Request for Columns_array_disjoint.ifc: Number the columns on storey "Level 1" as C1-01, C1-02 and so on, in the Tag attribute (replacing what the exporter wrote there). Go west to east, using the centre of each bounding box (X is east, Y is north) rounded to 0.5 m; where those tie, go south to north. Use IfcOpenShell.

First a look at what the model holds.

```python
import ifcopenshell
import ifcopenshell.util.element
import ifcopenshell.util.placement

model = ifcopenshell.open("Columns_array_disjoint.ifc")
print(model.schema)
storey = next(s for s in model.by_type("IfcBuildingStorey") if s.Name == "Level 1")
columns = [e for e in ifcopenshell.util.element.get_decomposition(storey) if e.is_a("IfcColumn")]
for e in sorted(columns, key=lambda e: e.id()):
    origin = ifcopenshell.util.placement.get_local_placement(e.ObjectPlacement)[:3, 3]
    print(e.id(), e.Tag, e.Name, origin.round(2) + 0.0, sep=" | ")
```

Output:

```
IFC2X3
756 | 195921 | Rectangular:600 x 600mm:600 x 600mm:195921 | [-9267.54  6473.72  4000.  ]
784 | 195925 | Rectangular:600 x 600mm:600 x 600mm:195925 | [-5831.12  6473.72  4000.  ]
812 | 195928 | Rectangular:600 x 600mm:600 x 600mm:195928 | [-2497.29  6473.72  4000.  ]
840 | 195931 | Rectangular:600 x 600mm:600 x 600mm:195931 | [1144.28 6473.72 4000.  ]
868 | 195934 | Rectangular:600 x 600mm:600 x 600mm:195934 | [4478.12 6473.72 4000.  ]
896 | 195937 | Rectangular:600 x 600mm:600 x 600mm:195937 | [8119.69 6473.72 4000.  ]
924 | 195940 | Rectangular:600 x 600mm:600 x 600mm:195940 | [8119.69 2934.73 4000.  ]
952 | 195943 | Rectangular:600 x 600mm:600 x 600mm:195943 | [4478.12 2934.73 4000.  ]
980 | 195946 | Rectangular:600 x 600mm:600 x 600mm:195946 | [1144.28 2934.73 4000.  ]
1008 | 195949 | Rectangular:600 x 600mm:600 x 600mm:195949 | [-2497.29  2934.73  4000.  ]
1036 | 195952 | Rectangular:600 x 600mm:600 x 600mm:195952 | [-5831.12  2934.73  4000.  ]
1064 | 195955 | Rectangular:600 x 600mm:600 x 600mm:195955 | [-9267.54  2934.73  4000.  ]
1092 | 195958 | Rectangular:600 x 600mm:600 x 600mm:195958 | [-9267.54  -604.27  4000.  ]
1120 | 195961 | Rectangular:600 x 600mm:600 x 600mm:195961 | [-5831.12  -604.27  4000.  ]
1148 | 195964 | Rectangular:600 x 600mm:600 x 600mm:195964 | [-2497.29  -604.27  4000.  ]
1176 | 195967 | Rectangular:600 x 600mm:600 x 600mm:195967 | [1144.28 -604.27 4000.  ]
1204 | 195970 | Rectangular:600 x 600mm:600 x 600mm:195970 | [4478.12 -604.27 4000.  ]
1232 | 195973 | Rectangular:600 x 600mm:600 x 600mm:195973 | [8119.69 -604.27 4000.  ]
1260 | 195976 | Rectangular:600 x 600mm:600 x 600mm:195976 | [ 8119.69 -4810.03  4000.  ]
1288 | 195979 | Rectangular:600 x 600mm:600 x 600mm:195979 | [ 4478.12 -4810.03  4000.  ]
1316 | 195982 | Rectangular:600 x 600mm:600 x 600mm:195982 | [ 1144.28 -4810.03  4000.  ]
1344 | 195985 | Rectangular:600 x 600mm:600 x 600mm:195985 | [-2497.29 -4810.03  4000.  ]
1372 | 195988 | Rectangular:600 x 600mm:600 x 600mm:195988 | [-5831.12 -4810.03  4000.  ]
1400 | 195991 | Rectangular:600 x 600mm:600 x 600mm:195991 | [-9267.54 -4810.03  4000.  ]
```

```python
import ifcopenshell
import ifcopenshell.geom
import ifcopenshell.util.element
import ifcopenshell.util.shape

model = ifcopenshell.open("Columns_array_disjoint.ifc")
settings = ifcopenshell.geom.settings()
settings.set("use-world-coords", True)


def centre(element):
    shape = ifcopenshell.geom.create_shape(settings, element)
    return ifcopenshell.util.shape.get_bbox_centroid(shape.geometry)


storey = next(s for s in model.by_type("IfcBuildingStorey") if s.Name == "Level 1")
columns = [e for e in ifcopenshell.util.element.get_decomposition(storey) if e.is_a("IfcColumn")]

# Insertion points can sit at a corner or the storey origin, so sort by the geometry (in metres).
centres = {e: centre(e) for e in columns}
columns.sort(key=lambda e: (round(centres[e][0] / 0.5), centres[e][1]))

for i, e in enumerate(columns, start=1):
    number = f"C1-{i:02d}"
    e.Tag = number
    print(e.id(), number)

model.write("Columns_array_disjoint_edited.ifc")
```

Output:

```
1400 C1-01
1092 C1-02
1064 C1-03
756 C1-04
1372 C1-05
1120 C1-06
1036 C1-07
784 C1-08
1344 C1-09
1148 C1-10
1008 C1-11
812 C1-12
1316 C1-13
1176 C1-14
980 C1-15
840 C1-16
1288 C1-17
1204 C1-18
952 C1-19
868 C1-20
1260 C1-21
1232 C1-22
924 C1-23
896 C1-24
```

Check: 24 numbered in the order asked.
